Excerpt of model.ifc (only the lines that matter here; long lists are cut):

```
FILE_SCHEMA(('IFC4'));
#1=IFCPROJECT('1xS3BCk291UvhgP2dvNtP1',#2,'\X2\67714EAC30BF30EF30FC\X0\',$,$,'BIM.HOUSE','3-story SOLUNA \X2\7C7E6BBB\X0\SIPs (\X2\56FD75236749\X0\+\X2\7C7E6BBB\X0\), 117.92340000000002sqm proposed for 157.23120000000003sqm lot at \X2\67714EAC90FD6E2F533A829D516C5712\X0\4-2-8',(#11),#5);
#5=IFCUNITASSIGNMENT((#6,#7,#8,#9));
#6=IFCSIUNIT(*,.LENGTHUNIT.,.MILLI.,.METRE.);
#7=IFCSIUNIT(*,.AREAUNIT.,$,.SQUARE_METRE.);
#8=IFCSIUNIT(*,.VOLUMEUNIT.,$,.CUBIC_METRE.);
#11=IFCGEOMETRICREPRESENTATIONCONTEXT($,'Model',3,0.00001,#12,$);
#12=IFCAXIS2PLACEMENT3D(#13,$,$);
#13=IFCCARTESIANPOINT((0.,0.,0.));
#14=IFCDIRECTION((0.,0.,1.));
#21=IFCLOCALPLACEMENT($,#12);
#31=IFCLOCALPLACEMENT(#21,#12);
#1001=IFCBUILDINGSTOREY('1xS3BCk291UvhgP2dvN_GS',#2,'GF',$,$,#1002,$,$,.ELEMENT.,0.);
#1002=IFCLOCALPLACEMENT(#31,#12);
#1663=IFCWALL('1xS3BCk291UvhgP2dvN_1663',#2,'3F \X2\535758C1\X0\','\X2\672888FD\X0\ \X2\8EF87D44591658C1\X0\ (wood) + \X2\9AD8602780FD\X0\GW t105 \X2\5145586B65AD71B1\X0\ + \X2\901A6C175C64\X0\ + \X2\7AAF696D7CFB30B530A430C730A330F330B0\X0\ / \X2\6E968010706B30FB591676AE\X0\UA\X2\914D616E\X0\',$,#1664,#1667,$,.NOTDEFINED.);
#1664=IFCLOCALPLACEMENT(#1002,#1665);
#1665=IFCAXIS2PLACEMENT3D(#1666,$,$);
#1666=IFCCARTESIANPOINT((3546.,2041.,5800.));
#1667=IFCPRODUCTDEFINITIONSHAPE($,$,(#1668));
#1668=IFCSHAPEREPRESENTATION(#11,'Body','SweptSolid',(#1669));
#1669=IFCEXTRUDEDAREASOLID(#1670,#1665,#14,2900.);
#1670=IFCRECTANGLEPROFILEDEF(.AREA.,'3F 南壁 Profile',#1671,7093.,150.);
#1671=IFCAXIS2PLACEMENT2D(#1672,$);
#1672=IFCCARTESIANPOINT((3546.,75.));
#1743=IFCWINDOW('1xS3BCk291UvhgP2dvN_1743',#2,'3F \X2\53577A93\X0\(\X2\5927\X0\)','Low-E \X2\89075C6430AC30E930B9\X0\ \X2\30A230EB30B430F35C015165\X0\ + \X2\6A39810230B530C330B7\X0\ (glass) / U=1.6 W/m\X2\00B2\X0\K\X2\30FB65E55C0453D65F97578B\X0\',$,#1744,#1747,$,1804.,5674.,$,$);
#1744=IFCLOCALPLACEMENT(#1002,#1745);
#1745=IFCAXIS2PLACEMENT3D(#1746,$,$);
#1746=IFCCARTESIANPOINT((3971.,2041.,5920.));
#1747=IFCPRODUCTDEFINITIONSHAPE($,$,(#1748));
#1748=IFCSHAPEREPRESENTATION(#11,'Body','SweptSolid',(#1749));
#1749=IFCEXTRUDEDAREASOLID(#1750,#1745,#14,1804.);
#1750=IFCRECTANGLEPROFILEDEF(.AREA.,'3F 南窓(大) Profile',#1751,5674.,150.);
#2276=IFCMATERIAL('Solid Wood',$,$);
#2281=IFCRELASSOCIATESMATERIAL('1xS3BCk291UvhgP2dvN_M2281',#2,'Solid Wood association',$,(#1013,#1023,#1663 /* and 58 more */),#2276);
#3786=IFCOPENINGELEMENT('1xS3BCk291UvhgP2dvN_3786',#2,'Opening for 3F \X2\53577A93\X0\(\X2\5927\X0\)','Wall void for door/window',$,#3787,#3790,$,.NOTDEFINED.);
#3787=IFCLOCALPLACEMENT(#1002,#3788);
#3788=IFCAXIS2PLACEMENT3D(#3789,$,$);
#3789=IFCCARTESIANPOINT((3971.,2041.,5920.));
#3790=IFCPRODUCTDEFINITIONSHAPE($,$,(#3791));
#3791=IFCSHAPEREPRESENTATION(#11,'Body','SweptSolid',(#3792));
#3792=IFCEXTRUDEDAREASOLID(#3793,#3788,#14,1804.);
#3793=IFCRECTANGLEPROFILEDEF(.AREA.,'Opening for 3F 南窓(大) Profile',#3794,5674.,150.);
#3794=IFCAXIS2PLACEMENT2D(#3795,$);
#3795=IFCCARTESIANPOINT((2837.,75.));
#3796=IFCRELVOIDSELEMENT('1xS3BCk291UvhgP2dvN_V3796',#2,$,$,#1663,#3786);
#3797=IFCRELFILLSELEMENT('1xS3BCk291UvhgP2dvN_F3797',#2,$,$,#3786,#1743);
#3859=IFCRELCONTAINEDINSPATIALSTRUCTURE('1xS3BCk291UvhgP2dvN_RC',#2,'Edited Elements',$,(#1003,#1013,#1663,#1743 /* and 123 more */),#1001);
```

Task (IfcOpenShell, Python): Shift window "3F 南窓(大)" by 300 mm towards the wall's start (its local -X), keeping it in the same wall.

```python
import ifcopenshell
import ifcopenshell.api.geometry
import ifcopenshell.util.placement
import ifcopenshell.util.unit

model = ifcopenshell.open("model.ifc")
unit_scale = ifcopenshell.util.unit.calculate_unit_scale(model)

window = model.by_id(1743)
opening = window.FillsVoids[0].RelatingOpeningElement
wall = opening.VoidsElements[0].RelatingBuildingElement

wall_matrix = ifcopenshell.util.placement.get_local_placement(wall.ObjectPlacement)
shift = wall_matrix[:3, 0] * -0.3 / unit_scale
before = ifcopenshell.util.placement.get_local_placement(window.ObjectPlacement)[:3, 3].copy()

# The window is not placed relative to its opening, so move both.
for product in (opening, window):
    matrix = ifcopenshell.util.placement.get_local_placement(product.ObjectPlacement)
    matrix[:3, 3] += shift
    ifcopenshell.api.geometry.edit_object_placement(model, product=product, matrix=matrix, is_si=False)

after = ifcopenshell.util.placement.get_local_placement(window.ObjectPlacement)[:3, 3]
print("window moved by", (after - before).round(3) + 0.0)

model.write("model_updated.ifc")
```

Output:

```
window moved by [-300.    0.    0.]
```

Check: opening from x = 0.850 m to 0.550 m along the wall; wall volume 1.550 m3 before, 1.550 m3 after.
